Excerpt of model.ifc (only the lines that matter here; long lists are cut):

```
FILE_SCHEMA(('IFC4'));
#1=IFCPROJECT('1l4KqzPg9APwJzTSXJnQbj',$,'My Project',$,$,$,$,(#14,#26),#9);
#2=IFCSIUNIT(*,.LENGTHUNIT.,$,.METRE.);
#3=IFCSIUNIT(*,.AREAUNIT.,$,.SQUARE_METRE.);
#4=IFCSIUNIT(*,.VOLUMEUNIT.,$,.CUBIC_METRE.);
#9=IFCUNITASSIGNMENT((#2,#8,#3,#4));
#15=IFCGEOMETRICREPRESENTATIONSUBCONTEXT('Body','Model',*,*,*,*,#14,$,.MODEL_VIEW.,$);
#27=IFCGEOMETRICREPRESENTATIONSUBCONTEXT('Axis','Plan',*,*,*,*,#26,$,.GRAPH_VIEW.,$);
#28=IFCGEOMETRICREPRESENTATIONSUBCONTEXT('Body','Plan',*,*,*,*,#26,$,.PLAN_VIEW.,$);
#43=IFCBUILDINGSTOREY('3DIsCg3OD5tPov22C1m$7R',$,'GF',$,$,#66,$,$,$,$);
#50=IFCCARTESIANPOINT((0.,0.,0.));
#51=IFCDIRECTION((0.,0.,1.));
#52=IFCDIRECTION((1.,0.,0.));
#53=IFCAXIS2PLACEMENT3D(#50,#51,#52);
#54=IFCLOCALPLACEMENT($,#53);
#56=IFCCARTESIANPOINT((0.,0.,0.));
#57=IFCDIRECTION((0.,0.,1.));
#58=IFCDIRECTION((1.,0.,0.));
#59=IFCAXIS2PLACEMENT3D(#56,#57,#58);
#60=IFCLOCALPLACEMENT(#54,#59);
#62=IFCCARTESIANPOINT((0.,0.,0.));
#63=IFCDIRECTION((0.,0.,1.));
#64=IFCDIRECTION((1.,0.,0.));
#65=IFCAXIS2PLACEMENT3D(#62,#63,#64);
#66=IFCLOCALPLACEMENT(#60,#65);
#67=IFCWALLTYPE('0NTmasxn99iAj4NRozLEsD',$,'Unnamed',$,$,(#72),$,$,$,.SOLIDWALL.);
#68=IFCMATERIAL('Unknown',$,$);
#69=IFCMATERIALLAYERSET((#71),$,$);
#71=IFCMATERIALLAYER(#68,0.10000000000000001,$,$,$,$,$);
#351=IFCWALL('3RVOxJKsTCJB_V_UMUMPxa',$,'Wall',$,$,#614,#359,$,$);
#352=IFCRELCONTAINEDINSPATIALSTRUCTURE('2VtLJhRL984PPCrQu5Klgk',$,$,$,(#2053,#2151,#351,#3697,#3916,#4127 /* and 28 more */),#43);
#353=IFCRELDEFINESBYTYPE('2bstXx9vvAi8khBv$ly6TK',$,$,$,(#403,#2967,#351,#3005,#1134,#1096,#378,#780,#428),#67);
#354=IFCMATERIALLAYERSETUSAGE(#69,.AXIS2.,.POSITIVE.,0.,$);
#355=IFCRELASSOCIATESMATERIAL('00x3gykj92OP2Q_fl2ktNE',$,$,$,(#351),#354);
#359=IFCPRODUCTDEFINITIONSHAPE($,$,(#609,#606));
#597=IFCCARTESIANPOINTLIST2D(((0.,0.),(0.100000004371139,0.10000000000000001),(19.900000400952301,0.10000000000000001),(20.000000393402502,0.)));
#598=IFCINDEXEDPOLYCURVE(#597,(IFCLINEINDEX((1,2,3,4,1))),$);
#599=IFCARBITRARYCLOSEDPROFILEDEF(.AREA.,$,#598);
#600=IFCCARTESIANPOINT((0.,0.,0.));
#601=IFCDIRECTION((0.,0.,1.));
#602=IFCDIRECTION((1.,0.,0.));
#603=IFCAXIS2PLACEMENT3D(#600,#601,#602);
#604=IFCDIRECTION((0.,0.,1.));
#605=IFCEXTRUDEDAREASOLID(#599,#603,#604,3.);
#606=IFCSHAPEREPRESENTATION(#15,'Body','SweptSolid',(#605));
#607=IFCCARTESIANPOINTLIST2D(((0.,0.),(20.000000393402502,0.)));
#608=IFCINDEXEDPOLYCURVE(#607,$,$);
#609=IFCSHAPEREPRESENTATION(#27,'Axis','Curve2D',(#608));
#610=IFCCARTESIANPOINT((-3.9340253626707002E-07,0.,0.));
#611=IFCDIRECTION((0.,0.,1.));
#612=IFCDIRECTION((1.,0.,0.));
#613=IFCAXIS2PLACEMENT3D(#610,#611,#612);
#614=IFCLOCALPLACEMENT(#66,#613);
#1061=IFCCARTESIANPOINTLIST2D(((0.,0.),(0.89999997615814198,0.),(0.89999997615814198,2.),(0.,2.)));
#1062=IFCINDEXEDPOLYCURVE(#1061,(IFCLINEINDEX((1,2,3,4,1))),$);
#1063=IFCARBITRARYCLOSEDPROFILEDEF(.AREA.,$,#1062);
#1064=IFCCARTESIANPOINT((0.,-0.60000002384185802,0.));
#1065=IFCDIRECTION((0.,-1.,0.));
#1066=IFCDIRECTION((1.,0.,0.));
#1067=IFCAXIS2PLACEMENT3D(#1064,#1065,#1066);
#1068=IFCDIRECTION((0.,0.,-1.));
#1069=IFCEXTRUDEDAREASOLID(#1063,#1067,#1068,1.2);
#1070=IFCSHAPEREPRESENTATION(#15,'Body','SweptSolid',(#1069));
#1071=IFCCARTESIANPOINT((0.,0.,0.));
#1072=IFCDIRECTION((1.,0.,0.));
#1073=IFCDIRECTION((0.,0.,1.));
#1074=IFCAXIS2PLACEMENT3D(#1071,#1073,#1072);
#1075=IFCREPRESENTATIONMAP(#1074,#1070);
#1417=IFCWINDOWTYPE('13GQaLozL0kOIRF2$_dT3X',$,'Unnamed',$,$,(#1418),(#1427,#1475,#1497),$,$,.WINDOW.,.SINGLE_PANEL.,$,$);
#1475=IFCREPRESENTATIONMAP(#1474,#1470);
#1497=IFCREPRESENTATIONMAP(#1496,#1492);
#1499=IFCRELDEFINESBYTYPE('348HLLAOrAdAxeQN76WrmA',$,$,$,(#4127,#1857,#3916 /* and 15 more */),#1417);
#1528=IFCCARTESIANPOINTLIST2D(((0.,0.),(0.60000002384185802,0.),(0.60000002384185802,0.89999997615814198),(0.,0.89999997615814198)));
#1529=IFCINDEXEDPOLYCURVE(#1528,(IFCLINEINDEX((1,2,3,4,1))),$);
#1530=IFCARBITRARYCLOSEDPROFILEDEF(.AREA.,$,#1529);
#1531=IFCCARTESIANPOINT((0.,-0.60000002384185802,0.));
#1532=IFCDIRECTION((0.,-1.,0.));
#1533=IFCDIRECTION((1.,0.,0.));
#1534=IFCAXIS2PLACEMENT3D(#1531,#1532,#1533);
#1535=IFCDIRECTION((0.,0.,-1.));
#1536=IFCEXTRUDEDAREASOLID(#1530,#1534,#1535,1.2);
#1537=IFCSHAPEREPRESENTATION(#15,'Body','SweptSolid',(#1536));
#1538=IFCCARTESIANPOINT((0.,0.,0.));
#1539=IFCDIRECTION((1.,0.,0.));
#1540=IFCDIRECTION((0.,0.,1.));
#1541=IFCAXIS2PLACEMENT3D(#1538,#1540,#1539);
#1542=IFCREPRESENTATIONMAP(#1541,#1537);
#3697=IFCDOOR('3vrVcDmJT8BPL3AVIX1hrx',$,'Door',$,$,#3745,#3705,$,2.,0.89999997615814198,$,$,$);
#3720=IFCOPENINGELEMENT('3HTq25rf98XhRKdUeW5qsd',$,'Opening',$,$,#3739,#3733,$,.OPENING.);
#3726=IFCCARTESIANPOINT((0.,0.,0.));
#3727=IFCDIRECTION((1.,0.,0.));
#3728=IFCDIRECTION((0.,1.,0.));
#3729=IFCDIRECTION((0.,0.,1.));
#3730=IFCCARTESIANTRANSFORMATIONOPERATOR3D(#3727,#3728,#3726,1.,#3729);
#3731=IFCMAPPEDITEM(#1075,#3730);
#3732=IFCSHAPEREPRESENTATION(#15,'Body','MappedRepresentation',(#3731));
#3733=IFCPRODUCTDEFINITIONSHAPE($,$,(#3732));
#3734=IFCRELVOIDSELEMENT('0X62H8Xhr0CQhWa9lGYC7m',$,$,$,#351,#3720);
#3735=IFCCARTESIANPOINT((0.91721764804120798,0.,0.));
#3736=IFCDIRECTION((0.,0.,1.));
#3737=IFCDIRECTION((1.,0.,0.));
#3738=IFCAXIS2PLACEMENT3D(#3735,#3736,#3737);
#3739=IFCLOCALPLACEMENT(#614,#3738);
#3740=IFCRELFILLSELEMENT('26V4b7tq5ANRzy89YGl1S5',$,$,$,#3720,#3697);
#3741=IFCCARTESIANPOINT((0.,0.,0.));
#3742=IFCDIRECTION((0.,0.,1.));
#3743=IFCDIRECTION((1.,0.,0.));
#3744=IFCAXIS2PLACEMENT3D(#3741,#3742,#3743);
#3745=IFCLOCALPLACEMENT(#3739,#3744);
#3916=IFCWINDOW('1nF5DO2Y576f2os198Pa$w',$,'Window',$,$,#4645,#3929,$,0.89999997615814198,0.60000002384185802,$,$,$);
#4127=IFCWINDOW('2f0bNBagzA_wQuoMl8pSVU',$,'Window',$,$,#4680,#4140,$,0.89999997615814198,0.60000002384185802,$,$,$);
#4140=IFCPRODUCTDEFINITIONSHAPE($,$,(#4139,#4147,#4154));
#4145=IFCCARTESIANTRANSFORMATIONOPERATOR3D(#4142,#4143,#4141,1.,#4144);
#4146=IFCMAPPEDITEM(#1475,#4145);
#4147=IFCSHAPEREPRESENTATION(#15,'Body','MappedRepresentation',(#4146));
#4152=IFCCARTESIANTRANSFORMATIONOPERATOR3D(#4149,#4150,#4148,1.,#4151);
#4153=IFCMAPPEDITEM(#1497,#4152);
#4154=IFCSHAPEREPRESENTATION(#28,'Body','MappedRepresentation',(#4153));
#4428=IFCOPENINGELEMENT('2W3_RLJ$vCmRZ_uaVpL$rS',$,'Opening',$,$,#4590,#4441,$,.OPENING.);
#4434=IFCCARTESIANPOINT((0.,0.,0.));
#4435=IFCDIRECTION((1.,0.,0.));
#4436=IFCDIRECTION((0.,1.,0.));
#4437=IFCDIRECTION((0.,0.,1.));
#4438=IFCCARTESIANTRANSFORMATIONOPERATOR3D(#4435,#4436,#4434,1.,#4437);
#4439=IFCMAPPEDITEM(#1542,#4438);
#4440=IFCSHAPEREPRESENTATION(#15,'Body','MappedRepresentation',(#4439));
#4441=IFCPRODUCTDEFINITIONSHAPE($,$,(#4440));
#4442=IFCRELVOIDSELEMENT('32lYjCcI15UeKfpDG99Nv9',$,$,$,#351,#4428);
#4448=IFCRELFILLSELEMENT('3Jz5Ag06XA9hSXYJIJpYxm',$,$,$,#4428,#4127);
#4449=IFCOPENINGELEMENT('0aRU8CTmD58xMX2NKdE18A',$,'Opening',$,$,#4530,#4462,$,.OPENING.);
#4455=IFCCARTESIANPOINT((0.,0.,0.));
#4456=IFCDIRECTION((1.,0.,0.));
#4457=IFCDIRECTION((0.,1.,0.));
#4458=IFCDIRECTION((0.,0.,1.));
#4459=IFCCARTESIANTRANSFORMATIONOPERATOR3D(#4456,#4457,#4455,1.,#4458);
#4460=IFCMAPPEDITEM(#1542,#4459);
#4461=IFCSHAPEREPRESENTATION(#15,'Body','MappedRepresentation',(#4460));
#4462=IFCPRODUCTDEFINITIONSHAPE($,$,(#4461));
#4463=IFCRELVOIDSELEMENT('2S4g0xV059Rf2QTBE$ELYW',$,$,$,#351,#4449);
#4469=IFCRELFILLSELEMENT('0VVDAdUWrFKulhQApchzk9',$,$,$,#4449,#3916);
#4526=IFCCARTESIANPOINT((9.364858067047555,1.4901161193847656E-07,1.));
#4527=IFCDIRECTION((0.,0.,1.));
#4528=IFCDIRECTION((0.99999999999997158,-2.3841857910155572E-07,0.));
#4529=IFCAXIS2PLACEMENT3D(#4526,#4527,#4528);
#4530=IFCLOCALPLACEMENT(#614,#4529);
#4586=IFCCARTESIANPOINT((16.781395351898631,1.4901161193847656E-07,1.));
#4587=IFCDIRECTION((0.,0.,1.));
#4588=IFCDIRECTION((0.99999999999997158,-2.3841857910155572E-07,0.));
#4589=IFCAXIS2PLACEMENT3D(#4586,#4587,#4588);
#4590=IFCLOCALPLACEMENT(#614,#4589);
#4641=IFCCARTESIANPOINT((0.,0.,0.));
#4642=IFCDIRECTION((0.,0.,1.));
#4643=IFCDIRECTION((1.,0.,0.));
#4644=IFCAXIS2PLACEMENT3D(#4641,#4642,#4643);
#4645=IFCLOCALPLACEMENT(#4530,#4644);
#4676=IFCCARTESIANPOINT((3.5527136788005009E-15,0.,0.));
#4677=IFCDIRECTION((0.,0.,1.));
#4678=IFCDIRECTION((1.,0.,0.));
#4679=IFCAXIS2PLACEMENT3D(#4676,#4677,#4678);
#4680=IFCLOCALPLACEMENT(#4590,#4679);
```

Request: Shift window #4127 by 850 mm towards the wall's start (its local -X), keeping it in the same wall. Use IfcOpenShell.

```python
import ifcopenshell
import ifcopenshell.api.geometry
import ifcopenshell.util.placement
import ifcopenshell.util.unit

model = ifcopenshell.open("model.ifc")
unit_scale = ifcopenshell.util.unit.calculate_unit_scale(model)

window = model.by_guid("2f0bNBagzA_wQuoMl8pSVU")
opening = window.FillsVoids[0].RelatingOpeningElement
wall = opening.VoidsElements[0].RelatingBuildingElement

wall_matrix = ifcopenshell.util.placement.get_local_placement(wall.ObjectPlacement)
shift = wall_matrix[:3, 0] * -0.85 / unit_scale
before = ifcopenshell.util.placement.get_local_placement(window.ObjectPlacement)[:3, 3].copy()

# The window is placed relative to its opening, so it follows when the opening moves.
matrix = ifcopenshell.util.placement.get_local_placement(opening.ObjectPlacement)
matrix[:3, 3] += shift
ifcopenshell.api.geometry.edit_object_placement(
    model, product=opening, matrix=matrix, is_si=False, should_transform_children=True
)

after = ifcopenshell.util.placement.get_local_placement(window.ObjectPlacement)[:3, 3]
print("window moved by", (after - before).round(3) + 0.0)

model.write("model_updated.ifc")
```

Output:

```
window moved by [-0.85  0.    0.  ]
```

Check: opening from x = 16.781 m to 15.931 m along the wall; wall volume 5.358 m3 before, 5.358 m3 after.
